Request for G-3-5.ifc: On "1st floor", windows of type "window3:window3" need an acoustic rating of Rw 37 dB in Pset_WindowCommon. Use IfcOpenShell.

First a look at what the model holds.

```python
import ifcopenshell
import ifcopenshell.util.element

model = ifcopenshell.open("G-3-5.ifc")
print(model.schema)
storey = next(s for s in model.by_type("IfcBuildingStorey") if s.Name == "1st floor")
windows = [e for e in ifcopenshell.util.element.get_decomposition(storey) if e.is_a("IfcWindow")]
seen = {}
for e in windows:
    element_type = ifcopenshell.util.element.get_type(e)
    key = (element_type.Name if element_type != e and element_type else None, ifcopenshell.util.element.get_pset(e, "Pset_WindowCommon", "AcousticRating"))
    seen[key] = seen.get(key, 0) + 1
for (name, value), count in sorted(seen.items(), key=str):
    print(count, "x", name, "|", value)
```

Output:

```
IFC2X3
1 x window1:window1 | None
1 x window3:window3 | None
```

```python
import ifcopenshell
import ifcopenshell.api.pset
import ifcopenshell.util.element

model = ifcopenshell.open("G-3-5.ifc")

storey = next(s for s in model.by_type("IfcBuildingStorey") if s.Name == "1st floor")
windows = [e for e in ifcopenshell.util.element.get_decomposition(storey) if e.is_a("IfcWindow")]

count = 0
for e in windows:
    element_type = ifcopenshell.util.element.get_type(e)
    if element_type in (None, e) or element_type.Name != "window3:window3":
        continue
    # add_pset returns the element's existing set when there is one.
    pset = ifcopenshell.api.pset.add_pset(model, product=e, name="Pset_WindowCommon")
    ifcopenshell.api.pset.edit_pset(model, pset=pset, properties={"AcousticRating": "Rw 37 dB"})
    count += 1

print(count, "windows updated")

model.write("G-3-5_v2.ifc")
```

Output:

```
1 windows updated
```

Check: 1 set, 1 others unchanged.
